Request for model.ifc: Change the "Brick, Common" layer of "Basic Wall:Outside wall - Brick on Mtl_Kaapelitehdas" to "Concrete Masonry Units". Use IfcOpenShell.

First a look at what the model holds.

```python
import ifcopenshell
import ifcopenshell.util.element

model = ifcopenshell.open("model.ifc")
print(model.schema)
for layer_set in model.by_type("IfcMaterialLayerSet"):
    if layer_set.LayerSetName == "Basic Wall:Outside wall - Brick on Mtl_Kaapelitehdas":
        for layer in layer_set.MaterialLayers:
            print(layer.id(), layer.Material and layer.Material.Name, layer.LayerThickness, sep=" | ")
        print(len(ifcopenshell.util.element.get_elements_by_material(model, layer_set)), "elements and types use it")
print(sorted(m.Name for m in model.by_type("IfcMaterial") if m.Name)[:60])
```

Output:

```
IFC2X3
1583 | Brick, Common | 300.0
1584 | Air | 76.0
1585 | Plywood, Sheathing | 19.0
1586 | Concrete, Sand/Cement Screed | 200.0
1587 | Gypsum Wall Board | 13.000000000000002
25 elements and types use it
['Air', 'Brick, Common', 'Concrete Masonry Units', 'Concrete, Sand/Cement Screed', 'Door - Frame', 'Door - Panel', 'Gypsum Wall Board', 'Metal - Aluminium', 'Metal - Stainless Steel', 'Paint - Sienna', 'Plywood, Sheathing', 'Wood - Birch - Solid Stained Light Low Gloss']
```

```python
import ifcopenshell
import ifcopenshell.api.material

model = ifcopenshell.open("model.ifc")

layer_set = next(s for s in model.by_type("IfcMaterialLayerSet") if s.LayerSetName == "Basic Wall:Outside wall - Brick on Mtl_Kaapelitehdas")
layer = next(l for l in layer_set.MaterialLayers if l.Material and l.Material.Name == "Brick, Common")
material = next(m for m in model.by_type("IfcMaterial") if m.Name == "Concrete Masonry Units")

# Point this one layer at the other material; renaming the old one would change it everywhere.
ifcopenshell.api.material.edit_layer(model, layer=layer, attributes={}, material=material)

print([l.Material.Name if l.Material else None for l in layer_set.MaterialLayers])

model.write("model_v2.ifc")
```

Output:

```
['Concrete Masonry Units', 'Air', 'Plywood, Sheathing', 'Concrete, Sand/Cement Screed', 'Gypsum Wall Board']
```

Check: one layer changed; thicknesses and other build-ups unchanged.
